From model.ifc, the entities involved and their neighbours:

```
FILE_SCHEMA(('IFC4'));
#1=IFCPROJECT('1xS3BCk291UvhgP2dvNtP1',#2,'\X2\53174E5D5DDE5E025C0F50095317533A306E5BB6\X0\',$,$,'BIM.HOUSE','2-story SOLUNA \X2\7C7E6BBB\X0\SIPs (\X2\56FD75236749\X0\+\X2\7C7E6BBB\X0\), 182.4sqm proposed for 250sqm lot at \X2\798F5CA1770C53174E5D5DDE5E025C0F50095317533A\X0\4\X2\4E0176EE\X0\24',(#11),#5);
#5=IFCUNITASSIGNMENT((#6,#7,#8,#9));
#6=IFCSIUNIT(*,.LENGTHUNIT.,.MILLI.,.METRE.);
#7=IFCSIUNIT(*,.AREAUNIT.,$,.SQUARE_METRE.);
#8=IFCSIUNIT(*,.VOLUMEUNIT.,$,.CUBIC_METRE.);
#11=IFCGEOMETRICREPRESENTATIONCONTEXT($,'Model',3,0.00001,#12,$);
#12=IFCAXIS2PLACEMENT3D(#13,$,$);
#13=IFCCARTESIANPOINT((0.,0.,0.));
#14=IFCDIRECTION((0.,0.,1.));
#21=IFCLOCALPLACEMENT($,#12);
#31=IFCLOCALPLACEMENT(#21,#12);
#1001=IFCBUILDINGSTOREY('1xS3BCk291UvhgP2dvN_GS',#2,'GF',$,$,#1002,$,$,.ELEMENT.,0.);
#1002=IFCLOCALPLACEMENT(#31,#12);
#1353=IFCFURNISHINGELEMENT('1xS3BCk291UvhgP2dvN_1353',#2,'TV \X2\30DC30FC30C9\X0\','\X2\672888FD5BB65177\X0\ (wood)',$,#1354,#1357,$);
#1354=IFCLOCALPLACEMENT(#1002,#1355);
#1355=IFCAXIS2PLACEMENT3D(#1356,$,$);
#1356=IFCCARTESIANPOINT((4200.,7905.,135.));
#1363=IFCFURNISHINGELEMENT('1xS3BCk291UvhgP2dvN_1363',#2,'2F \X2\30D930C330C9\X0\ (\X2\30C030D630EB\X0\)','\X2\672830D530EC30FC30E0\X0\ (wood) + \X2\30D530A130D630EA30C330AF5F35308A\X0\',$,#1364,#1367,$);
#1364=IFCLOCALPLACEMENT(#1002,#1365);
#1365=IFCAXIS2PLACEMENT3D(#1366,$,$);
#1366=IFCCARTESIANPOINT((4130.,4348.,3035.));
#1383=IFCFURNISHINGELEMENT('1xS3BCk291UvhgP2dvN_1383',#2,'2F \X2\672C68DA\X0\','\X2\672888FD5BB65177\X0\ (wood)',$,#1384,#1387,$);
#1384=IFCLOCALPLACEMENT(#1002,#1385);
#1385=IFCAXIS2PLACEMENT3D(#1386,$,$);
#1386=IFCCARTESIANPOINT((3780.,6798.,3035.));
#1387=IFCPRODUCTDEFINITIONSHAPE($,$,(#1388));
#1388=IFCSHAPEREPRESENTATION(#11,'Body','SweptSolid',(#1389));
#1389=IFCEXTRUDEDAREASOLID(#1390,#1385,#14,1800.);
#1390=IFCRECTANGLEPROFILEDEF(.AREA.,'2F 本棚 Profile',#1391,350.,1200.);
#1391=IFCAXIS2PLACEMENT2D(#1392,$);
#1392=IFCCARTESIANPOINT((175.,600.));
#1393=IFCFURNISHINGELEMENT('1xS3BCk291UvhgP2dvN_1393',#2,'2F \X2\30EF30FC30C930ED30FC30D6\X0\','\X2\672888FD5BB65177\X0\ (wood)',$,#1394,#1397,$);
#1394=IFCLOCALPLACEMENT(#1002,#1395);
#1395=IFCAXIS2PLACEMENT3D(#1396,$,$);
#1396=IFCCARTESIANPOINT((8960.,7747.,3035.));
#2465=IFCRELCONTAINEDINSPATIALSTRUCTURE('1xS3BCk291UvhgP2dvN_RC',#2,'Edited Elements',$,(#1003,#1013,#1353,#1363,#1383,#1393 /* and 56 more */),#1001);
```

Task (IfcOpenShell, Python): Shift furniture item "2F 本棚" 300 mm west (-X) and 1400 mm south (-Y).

```python
import ifcopenshell
import ifcopenshell.api.geometry
import ifcopenshell.util.placement

model = ifcopenshell.open("model.ifc")

item = model.by_guid("1xS3BCk291UvhgP2dvN_1383")
matrix = ifcopenshell.util.placement.get_local_placement(item.ObjectPlacement)
matrix[0, 3] -= 300.0
matrix[1, 3] -= 1400.0
ifcopenshell.api.geometry.edit_object_placement(model, product=item, matrix=matrix, is_si=False)

print(ifcopenshell.util.placement.get_local_placement(item.ObjectPlacement).round(3) + 0.0)

model.write("model_edited.ifc")
```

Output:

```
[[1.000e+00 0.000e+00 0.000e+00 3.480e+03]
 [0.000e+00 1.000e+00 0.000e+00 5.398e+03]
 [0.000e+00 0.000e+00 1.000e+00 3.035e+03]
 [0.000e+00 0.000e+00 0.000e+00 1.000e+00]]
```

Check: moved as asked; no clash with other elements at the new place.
